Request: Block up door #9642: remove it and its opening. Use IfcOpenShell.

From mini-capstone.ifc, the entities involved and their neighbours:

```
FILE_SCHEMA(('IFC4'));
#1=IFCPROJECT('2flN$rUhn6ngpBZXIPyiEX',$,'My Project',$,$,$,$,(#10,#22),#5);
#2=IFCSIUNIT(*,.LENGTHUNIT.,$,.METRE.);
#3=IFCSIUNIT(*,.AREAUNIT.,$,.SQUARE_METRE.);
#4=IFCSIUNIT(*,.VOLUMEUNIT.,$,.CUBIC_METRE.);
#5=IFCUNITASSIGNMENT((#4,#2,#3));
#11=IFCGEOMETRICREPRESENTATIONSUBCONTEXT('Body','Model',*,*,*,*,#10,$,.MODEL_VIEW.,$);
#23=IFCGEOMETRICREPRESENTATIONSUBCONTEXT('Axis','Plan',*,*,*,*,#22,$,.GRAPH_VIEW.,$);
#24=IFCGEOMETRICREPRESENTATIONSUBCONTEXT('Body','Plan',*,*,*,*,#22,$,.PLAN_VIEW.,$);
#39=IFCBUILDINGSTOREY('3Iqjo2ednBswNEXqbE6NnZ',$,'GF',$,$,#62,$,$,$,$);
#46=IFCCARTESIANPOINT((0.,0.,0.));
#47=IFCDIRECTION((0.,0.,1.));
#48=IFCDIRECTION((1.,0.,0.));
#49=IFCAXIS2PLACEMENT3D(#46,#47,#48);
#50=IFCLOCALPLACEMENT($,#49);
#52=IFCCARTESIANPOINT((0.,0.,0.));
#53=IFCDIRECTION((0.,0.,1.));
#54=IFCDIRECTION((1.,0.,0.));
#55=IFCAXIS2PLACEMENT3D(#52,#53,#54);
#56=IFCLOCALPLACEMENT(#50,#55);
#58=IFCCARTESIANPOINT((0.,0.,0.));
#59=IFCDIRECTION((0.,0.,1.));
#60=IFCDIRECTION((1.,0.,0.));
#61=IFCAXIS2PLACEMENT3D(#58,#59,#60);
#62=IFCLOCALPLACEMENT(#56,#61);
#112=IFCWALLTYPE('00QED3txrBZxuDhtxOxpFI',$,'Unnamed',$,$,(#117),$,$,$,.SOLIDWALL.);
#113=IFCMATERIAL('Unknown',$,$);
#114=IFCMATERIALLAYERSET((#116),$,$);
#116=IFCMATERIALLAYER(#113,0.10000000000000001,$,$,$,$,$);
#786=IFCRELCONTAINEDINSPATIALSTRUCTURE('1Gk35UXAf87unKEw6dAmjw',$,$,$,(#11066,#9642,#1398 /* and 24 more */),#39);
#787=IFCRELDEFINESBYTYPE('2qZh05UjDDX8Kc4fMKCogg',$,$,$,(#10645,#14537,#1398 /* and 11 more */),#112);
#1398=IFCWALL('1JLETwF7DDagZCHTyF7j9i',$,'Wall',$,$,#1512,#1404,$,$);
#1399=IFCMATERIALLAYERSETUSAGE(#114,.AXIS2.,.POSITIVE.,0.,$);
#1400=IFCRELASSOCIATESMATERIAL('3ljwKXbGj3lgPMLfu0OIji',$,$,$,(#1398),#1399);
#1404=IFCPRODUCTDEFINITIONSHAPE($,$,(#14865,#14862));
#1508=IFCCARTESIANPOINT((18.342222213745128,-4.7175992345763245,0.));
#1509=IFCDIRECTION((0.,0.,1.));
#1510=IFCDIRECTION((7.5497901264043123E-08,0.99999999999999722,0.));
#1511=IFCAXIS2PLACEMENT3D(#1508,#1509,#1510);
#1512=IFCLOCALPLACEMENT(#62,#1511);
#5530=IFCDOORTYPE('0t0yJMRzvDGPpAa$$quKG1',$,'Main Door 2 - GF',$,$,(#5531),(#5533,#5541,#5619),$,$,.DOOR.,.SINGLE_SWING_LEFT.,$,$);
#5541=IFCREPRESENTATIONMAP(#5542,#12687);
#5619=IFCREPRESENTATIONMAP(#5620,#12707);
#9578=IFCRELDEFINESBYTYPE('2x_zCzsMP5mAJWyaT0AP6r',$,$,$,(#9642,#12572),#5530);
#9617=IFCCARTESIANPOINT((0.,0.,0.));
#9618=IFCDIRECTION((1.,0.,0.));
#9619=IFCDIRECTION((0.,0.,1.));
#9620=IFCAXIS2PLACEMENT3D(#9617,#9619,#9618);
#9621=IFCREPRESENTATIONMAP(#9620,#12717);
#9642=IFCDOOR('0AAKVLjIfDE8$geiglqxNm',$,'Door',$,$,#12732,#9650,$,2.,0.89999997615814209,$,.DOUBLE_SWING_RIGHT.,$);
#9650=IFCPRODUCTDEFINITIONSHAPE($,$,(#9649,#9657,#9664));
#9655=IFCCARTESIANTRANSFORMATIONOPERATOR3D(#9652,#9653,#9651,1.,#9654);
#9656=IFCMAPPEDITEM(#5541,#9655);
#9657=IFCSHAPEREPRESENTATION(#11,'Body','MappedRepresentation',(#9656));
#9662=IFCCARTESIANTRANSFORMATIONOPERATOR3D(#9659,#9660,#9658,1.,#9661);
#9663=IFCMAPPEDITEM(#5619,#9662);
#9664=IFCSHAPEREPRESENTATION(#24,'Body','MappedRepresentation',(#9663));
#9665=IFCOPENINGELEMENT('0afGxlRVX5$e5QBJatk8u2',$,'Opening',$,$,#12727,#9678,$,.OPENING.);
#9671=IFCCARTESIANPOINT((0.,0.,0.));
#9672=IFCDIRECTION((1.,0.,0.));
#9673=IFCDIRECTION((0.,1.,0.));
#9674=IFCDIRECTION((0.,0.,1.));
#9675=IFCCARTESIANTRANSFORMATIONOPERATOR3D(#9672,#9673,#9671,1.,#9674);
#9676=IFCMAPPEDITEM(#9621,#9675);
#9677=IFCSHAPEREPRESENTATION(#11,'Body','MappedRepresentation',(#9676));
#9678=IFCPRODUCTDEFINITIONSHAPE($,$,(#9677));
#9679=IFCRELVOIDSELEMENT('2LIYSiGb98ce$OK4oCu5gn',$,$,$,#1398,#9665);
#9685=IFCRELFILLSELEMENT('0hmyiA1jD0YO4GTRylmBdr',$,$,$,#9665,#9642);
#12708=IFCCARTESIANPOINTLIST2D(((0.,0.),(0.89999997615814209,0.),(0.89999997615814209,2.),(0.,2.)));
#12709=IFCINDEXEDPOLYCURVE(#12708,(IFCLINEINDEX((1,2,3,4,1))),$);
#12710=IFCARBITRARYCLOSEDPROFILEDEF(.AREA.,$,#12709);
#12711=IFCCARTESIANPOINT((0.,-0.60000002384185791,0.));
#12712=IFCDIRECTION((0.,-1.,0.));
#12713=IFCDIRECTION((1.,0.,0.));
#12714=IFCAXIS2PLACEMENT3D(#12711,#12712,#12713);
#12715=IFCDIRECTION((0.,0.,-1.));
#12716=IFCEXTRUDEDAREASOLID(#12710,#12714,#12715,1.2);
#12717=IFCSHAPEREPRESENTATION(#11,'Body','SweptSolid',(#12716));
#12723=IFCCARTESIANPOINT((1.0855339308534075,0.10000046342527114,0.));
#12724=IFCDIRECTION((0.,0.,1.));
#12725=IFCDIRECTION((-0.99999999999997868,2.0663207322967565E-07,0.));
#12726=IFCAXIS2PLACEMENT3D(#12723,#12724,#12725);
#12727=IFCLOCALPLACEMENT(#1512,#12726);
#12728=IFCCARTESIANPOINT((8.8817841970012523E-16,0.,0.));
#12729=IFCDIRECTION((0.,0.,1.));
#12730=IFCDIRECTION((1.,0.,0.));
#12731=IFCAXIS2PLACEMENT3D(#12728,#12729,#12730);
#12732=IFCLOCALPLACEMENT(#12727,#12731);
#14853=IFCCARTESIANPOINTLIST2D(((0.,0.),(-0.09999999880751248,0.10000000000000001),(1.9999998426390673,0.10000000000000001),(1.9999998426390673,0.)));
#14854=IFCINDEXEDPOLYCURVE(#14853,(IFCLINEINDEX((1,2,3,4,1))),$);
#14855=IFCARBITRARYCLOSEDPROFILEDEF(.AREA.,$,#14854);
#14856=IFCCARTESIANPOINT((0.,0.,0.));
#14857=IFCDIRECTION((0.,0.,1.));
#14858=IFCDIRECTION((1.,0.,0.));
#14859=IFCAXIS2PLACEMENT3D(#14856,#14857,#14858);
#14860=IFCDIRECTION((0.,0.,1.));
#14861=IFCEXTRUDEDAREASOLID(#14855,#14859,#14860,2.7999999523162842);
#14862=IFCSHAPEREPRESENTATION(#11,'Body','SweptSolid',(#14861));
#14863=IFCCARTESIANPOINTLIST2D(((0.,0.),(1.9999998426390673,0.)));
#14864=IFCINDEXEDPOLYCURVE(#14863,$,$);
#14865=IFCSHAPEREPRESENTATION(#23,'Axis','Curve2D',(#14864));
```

```python
import ifcopenshell
import ifcopenshell.api.feature
import ifcopenshell.api.root
import ifcopenshell.geom
import ifcopenshell.util.shape

model = ifcopenshell.open("mini-capstone.ifc")
settings = ifcopenshell.geom.settings()


def volume(element):
    """Net volume in cubic metres, openings subtracted."""
    shape = ifcopenshell.geom.create_shape(settings, element)
    return ifcopenshell.util.shape.get_volume(shape.geometry)


door = model.by_id(9642)
opening = door.FillsVoids[0].RelatingOpeningElement
wall = opening.VoidsElements[0].RelatingBuildingElement
before = volume(wall)

ifcopenshell.api.root.remove_product(model, product=door)
ifcopenshell.api.feature.remove_feature(model, feature=opening)

after = volume(wall)

print(f"wall volume {before:.3f} -> {after:.3f} m3")

model.write("mini-capstone_updated.ifc")
```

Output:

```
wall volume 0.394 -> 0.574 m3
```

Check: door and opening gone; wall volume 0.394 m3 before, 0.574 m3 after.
